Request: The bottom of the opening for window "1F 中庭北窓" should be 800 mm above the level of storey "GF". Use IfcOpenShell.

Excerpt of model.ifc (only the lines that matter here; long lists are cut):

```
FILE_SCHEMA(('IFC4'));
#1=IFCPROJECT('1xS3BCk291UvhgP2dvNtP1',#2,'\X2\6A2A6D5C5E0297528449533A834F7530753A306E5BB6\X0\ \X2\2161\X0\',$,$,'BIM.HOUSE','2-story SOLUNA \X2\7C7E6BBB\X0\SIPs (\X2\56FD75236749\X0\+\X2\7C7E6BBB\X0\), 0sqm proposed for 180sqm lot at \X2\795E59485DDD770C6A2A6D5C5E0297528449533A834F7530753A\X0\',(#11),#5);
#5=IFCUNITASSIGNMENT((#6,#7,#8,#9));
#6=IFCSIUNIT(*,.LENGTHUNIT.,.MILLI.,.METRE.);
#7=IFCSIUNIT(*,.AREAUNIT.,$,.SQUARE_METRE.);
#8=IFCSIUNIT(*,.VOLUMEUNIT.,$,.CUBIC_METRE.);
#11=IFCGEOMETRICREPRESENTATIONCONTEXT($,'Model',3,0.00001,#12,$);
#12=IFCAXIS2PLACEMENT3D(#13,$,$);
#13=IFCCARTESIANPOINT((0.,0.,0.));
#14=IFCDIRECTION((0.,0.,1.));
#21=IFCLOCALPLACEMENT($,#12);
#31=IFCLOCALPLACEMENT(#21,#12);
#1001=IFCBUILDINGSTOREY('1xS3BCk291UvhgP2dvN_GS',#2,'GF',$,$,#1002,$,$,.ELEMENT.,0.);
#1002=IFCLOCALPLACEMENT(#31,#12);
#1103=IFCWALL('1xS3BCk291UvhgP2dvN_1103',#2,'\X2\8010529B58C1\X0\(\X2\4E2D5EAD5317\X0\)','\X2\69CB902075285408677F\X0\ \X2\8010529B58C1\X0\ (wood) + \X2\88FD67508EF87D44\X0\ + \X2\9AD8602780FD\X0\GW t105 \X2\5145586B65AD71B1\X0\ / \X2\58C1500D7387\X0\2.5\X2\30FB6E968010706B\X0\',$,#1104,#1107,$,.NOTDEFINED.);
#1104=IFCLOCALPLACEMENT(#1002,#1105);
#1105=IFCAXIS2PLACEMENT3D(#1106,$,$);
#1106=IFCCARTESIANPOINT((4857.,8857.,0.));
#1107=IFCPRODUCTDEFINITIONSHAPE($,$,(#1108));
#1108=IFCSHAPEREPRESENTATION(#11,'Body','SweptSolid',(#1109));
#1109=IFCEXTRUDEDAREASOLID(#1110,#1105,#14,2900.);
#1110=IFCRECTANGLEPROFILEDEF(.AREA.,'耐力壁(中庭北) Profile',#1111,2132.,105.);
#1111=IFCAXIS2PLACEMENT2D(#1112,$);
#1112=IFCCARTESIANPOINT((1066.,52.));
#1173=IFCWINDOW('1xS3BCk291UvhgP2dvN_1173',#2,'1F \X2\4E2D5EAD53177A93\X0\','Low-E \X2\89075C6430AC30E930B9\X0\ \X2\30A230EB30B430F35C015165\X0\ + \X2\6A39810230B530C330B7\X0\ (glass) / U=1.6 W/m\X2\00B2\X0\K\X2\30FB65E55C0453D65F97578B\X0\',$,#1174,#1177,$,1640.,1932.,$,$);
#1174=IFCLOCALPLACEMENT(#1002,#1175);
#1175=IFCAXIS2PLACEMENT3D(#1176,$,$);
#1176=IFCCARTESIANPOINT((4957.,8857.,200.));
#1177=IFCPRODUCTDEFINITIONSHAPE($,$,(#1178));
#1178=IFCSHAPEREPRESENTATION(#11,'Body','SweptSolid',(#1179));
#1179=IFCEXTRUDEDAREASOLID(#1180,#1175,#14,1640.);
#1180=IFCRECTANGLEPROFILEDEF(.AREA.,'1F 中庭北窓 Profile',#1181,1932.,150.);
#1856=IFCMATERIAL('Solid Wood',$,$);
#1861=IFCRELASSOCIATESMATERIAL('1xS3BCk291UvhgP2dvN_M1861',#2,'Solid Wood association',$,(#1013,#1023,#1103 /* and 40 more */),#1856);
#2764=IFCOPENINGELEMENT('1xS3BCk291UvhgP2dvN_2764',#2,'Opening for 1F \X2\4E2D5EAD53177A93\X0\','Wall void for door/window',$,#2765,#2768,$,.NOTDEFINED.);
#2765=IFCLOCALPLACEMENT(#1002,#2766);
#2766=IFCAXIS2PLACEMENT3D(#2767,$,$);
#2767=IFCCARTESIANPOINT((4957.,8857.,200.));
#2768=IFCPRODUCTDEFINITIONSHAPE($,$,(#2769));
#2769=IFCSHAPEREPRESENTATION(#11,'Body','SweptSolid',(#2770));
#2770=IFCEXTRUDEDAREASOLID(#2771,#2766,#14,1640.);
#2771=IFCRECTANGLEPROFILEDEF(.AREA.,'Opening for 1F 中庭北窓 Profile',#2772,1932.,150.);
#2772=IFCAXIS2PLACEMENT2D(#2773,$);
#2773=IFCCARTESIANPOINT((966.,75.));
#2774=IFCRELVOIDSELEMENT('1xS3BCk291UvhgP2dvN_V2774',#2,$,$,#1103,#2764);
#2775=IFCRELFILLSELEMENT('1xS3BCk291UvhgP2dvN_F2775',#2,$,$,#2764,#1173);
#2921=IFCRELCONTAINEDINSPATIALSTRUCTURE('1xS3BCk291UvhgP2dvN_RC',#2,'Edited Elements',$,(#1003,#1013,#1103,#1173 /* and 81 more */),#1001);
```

```python
import numpy as np
import ifcopenshell
import ifcopenshell.api.geometry
import ifcopenshell.geom
import ifcopenshell.util.element
import ifcopenshell.util.placement
import ifcopenshell.util.shape
import ifcopenshell.util.unit

model = ifcopenshell.open("model.ifc")
unit_scale = ifcopenshell.util.unit.calculate_unit_scale(model)

window = model.by_guid("1xS3BCk291UvhgP2dvN_1173")
opening = window.FillsVoids[0].RelatingOpeningElement
storey = ifcopenshell.util.element.get_container(window, ifc_class="IfcBuildingStorey")
level = ifcopenshell.util.placement.get_local_placement(storey.ObjectPlacement)[2, 3]

# The opening's origin need not be at the sill, so measure its lowest point.
shape = ifcopenshell.geom.create_shape(ifcopenshell.geom.settings(), opening)
bottom = ifcopenshell.util.shape.get_shape_bottom_elevation(shape, shape.geometry) / unit_scale
dz = level + 0.8 / unit_scale - bottom

shift = np.array([0.0, 0.0, dz])
# The window is not placed relative to its opening, so move both.
for product in (opening, window):
    matrix = ifcopenshell.util.placement.get_local_placement(product.ObjectPlacement)
    matrix[:3, 3] += shift
    ifcopenshell.api.geometry.edit_object_placement(model, product=product, matrix=matrix, is_si=False)

print(f"moved by {dz * unit_scale:+.3f} m")

model.write("model_rev.ifc")
```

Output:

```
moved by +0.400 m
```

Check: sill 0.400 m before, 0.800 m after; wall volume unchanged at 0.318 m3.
